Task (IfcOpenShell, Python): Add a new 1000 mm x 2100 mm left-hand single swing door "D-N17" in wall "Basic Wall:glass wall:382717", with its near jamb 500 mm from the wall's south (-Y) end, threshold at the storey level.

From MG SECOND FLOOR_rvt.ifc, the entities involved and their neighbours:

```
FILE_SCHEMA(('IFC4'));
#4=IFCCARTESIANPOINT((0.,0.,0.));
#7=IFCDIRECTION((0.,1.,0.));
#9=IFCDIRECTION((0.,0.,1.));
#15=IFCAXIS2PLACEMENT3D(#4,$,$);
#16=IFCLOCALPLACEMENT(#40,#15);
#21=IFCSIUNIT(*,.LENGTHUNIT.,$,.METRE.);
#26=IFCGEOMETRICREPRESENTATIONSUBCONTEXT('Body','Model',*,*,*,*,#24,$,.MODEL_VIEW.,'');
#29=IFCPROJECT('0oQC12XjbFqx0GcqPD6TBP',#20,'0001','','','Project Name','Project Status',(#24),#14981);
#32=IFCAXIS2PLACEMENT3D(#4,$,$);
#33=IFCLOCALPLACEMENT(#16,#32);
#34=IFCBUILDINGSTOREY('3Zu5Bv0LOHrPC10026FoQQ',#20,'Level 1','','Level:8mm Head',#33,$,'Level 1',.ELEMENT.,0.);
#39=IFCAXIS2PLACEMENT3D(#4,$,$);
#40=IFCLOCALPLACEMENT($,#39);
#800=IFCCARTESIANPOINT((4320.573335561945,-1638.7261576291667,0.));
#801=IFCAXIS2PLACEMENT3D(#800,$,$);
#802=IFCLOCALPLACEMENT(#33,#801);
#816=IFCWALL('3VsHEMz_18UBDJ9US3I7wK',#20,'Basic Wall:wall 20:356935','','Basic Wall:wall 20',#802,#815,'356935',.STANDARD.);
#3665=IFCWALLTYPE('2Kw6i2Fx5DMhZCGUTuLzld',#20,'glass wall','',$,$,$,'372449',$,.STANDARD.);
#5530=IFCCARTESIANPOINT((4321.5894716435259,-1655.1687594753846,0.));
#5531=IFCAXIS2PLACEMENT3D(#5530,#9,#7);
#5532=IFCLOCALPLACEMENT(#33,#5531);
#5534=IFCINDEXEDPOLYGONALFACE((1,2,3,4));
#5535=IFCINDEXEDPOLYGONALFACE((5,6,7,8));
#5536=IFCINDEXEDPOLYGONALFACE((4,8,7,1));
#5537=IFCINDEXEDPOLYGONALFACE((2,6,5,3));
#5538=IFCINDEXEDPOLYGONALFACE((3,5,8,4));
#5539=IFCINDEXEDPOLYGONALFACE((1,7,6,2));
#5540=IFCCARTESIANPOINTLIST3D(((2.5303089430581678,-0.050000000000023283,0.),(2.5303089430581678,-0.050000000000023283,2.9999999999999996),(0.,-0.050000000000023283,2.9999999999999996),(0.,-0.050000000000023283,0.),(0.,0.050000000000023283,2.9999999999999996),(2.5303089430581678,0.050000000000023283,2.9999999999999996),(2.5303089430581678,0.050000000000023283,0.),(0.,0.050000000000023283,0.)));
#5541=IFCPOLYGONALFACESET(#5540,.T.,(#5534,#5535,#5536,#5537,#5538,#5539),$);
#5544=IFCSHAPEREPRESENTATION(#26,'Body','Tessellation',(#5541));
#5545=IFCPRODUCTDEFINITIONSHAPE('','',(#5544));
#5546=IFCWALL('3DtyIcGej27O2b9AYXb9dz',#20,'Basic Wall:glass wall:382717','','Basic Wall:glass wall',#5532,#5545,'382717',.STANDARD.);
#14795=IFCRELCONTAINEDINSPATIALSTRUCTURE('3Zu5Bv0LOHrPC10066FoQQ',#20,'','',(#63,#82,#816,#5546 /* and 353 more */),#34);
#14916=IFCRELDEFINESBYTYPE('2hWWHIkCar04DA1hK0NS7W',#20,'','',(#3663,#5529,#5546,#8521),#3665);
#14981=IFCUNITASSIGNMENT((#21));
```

```python
import numpy as np
import ifcopenshell
import ifcopenshell.api.feature
import ifcopenshell.api.geometry
import ifcopenshell.api.root
import ifcopenshell.api.spatial
import ifcopenshell.geom
import ifcopenshell.util.element
import ifcopenshell.util.placement
import ifcopenshell.util.representation
import ifcopenshell.util.shape
import ifcopenshell.util.unit

model = ifcopenshell.open("MG SECOND FLOOR_rvt.ifc")
unit_scale = ifcopenshell.util.unit.calculate_unit_scale(model)
settings = ifcopenshell.geom.settings()


def volume(element):
    """Net volume in cubic metres, openings subtracted."""
    shape = ifcopenshell.geom.create_shape(settings, element)
    return ifcopenshell.util.shape.get_volume(shape.geometry)


wall = model.by_guid("3DtyIcGej27O2b9AYXb9dz")
storey = ifcopenshell.util.element.get_container(wall, ifc_class="IfcBuildingStorey")
context = ifcopenshell.util.representation.get_context(model, "Model", "Body", "MODEL_VIEW")
before = volume(wall)

width, height, from_end, sill = 1, 2.1, 0.5, 0.0  # metres

# The wall runs along its own X axis, and the end named is its -X end.
wall_shape = ifcopenshell.geom.create_shape(settings, wall)
x, y, z = ifcopenshell.util.shape.get_vertices(wall_shape.geometry).T
start = x.min() + from_end
face, thickness = float(y.min()), float(y.max() - y.min())
wall_matrix = ifcopenshell.util.placement.get_local_placement(wall.ObjectPlacement)
level = ifcopenshell.util.placement.get_local_placement(storey.ObjectPlacement)[2, 3]


def in_wall(x, y):
    """Placement at x, y metres in the wall's axes, at sill height."""
    matrix = wall_matrix.copy()
    matrix[:, 3] = wall_matrix @ np.array([x / unit_scale, y / unit_scale, 0.0, 1.0])
    matrix[2, 3] = level + sill / unit_scale
    return matrix


# Opening: a box that overshoots both wall faces by 50 mm.
opening = ifcopenshell.api.root.create_entity(model, ifc_class="IfcOpeningElement", predefined_type="OPENING")
box = ifcopenshell.api.geometry.add_wall_representation(
    model, context=context, length=width, height=height, thickness=thickness + 0.1
)
ifcopenshell.api.geometry.assign_representation(model, product=opening, representation=box)
ifcopenshell.api.geometry.edit_object_placement(model, product=opening, matrix=in_wall(start, face - 0.05), is_si=False)
ifcopenshell.api.feature.add_feature(model, feature=opening, element=wall)

door = ifcopenshell.api.root.create_entity(model, ifc_class="IfcDoor", name="D-N17", predefined_type="DOOR")
door.OverallWidth, door.OverallHeight = width / unit_scale, height / unit_scale
door.OperationType = "SINGLE_SWING_LEFT"
body = ifcopenshell.api.geometry.add_door_representation(
    model,
    context=context,
    overall_width=door.OverallWidth,
    overall_height=door.OverallHeight,
    operation_type="SINGLE_SWING_LEFT",
    lining_properties={"LiningDepth": thickness / unit_scale, "ThresholdDepth": thickness / unit_scale},
)
ifcopenshell.api.geometry.assign_representation(model, product=door, representation=body)
ifcopenshell.api.spatial.assign_container(model, products=[door], relating_structure=storey)
ifcopenshell.api.feature.add_filling(model, opening=opening, element=door)

# The lining spans the wall, so the door starts at the wall face.
ifcopenshell.api.geometry.edit_object_placement(model, product=door, matrix=in_wall(start, face), is_si=False)

after = volume(wall)

print(f"wall volume {before:.3f} -> {after:.3f} m3")

model.write("MG SECOND FLOOR_rvt_v2.ifc")
```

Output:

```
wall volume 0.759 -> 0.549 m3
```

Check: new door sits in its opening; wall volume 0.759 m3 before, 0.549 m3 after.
